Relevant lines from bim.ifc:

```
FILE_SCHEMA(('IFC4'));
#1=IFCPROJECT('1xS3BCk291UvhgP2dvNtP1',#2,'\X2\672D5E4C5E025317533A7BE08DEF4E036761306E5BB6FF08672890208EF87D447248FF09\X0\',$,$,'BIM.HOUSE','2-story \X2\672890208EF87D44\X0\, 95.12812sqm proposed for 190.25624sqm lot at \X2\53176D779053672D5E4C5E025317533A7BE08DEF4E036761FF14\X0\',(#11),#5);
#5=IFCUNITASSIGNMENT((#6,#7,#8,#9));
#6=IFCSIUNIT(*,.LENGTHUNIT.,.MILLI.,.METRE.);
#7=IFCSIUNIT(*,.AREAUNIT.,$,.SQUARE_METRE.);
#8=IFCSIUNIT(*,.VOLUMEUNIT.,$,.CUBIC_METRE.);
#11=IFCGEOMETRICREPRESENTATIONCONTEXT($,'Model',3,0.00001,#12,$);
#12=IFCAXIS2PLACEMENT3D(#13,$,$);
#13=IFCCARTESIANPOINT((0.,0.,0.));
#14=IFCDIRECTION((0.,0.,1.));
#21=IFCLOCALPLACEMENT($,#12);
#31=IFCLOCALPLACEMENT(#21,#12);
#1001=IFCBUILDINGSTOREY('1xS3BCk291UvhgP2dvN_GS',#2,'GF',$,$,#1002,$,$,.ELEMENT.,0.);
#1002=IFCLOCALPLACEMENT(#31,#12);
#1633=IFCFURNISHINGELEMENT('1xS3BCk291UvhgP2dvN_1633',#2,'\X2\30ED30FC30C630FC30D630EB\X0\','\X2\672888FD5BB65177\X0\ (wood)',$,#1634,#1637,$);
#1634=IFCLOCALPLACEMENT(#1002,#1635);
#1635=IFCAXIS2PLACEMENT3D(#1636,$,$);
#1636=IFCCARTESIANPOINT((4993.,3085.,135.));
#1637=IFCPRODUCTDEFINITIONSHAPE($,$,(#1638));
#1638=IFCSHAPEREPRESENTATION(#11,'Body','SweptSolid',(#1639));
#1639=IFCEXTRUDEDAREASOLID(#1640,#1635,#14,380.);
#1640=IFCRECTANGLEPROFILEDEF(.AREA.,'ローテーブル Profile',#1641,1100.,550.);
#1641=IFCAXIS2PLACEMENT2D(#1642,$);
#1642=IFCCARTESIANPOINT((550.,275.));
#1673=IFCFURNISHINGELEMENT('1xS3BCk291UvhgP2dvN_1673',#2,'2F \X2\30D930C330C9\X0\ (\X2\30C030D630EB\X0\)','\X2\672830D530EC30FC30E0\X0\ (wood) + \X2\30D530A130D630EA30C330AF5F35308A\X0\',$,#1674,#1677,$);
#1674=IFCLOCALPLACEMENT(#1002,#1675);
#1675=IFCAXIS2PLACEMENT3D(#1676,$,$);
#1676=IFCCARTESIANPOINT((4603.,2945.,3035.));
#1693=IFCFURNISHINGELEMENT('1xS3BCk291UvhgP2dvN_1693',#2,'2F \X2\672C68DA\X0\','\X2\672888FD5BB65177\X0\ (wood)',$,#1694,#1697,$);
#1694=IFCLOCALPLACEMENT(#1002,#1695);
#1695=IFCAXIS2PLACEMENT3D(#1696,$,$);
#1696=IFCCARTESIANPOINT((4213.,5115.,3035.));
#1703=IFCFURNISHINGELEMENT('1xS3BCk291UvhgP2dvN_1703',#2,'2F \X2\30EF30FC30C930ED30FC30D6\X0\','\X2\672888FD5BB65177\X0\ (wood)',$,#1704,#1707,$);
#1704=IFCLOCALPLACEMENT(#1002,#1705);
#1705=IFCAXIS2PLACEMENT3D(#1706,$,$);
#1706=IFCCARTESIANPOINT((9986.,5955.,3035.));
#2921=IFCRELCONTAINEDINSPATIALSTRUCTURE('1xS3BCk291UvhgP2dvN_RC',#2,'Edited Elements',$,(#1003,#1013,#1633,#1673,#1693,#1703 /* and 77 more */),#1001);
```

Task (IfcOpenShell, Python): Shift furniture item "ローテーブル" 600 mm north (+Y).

```python
import ifcopenshell
import ifcopenshell.api.geometry
import ifcopenshell.util.placement

model = ifcopenshell.open("bim.ifc")

item = model.by_id(1633)
matrix = ifcopenshell.util.placement.get_local_placement(item.ObjectPlacement)
matrix[1, 3] += 600.0
ifcopenshell.api.geometry.edit_object_placement(model, product=item, matrix=matrix, is_si=False)

print(ifcopenshell.util.placement.get_local_placement(item.ObjectPlacement).round(3) + 0.0)

model.write("bim-out.ifc")
```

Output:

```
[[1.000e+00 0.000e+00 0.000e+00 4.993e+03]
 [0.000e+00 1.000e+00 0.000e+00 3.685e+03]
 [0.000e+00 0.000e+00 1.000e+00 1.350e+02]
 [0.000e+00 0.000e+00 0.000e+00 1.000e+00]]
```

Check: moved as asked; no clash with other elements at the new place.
